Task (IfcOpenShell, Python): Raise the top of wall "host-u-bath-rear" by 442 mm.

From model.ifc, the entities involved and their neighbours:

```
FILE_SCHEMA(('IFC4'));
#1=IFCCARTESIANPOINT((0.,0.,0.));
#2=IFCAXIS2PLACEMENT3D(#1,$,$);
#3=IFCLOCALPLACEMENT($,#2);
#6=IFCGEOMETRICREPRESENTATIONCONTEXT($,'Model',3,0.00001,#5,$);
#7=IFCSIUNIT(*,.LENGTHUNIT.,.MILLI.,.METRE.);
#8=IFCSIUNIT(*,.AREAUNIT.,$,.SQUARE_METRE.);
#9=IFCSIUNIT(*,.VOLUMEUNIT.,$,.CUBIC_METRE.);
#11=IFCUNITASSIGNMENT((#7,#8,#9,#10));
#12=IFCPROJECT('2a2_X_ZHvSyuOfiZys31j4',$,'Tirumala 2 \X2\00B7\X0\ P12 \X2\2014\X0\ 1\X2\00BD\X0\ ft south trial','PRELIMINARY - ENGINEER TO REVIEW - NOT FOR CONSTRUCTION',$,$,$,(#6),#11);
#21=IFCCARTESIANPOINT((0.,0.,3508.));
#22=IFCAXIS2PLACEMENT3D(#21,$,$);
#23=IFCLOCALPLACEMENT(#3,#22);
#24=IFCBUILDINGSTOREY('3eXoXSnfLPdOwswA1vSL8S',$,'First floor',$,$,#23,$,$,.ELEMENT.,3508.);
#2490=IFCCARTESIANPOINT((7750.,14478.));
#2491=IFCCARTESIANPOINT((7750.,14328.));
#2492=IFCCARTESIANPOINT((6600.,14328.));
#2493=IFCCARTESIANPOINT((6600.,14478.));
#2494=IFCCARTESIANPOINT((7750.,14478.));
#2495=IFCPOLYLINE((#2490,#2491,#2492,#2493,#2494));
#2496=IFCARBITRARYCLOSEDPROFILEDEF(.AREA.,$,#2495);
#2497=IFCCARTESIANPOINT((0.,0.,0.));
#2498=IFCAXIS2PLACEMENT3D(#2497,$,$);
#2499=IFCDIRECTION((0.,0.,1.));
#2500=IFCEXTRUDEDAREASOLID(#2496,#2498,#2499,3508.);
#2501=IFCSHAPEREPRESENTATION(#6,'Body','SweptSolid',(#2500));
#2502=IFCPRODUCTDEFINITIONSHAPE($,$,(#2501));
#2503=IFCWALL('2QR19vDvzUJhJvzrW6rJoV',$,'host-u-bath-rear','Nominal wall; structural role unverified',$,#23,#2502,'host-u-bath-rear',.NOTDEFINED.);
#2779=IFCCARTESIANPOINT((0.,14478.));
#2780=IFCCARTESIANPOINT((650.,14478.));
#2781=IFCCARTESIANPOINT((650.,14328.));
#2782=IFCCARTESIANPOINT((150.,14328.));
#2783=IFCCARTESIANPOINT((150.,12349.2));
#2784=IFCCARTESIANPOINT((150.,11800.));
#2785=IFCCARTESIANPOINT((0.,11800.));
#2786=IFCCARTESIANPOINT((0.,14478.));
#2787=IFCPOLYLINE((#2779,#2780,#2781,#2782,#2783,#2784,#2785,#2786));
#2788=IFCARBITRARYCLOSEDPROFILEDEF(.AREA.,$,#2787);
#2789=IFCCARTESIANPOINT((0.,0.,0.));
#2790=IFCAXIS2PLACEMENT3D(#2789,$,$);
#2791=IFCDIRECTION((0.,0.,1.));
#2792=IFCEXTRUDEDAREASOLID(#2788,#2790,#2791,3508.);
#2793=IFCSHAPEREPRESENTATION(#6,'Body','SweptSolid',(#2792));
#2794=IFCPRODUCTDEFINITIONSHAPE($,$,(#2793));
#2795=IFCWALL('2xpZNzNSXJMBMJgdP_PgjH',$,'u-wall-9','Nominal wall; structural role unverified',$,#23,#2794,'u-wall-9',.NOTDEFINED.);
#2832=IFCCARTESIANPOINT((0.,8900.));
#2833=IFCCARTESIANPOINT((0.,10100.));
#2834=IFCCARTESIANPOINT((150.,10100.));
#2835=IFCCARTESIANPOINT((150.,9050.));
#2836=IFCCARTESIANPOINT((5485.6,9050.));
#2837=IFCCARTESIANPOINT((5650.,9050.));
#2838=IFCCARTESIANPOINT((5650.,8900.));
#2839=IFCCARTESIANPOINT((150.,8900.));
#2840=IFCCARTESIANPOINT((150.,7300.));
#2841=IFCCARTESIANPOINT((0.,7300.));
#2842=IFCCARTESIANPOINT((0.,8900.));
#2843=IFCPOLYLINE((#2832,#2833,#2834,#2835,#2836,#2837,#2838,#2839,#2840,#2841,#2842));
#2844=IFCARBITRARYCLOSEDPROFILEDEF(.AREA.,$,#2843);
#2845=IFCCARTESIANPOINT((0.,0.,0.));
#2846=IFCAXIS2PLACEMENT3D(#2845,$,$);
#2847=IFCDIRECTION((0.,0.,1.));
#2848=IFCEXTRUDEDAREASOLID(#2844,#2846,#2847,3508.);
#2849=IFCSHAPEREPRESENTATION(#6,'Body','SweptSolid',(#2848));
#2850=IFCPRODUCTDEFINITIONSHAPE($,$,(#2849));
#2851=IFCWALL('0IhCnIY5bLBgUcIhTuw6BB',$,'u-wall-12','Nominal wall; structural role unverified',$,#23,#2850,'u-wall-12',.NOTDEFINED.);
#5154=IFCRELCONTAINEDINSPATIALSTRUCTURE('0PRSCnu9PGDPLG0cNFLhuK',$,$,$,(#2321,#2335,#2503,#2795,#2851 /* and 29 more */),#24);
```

```python
import ifcopenshell
import ifcopenshell.geom
import ifcopenshell.util.shape
import ifcopenshell.util.unit

model = ifcopenshell.open("model.ifc")
unit_scale = ifcopenshell.util.unit.calculate_unit_scale(model)
settings = ifcopenshell.geom.settings()


def volume(element):
    """Net volume in cubic metres, openings subtracted."""
    shape = ifcopenshell.geom.create_shape(settings, element)
    return ifcopenshell.util.shape.get_volume(shape.geometry)


wall = model.by_guid("2QR19vDvzUJhJvzrW6rJoV")
before = volume(wall)

body = next(r for r in wall.Representation.Representations if r.RepresentationIdentifier == "Body")
solid = body.Items[0]
old_height = solid.Depth
solid.Depth += 0.442 / unit_scale
after = volume(wall)

print(f"height {old_height:g} -> {solid.Depth:g}, volume {before:.3f} -> {after:.3f} m3")

model.write("model_v2.ifc")
```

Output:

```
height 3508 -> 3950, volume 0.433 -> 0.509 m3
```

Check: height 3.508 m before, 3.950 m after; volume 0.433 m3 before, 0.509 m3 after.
